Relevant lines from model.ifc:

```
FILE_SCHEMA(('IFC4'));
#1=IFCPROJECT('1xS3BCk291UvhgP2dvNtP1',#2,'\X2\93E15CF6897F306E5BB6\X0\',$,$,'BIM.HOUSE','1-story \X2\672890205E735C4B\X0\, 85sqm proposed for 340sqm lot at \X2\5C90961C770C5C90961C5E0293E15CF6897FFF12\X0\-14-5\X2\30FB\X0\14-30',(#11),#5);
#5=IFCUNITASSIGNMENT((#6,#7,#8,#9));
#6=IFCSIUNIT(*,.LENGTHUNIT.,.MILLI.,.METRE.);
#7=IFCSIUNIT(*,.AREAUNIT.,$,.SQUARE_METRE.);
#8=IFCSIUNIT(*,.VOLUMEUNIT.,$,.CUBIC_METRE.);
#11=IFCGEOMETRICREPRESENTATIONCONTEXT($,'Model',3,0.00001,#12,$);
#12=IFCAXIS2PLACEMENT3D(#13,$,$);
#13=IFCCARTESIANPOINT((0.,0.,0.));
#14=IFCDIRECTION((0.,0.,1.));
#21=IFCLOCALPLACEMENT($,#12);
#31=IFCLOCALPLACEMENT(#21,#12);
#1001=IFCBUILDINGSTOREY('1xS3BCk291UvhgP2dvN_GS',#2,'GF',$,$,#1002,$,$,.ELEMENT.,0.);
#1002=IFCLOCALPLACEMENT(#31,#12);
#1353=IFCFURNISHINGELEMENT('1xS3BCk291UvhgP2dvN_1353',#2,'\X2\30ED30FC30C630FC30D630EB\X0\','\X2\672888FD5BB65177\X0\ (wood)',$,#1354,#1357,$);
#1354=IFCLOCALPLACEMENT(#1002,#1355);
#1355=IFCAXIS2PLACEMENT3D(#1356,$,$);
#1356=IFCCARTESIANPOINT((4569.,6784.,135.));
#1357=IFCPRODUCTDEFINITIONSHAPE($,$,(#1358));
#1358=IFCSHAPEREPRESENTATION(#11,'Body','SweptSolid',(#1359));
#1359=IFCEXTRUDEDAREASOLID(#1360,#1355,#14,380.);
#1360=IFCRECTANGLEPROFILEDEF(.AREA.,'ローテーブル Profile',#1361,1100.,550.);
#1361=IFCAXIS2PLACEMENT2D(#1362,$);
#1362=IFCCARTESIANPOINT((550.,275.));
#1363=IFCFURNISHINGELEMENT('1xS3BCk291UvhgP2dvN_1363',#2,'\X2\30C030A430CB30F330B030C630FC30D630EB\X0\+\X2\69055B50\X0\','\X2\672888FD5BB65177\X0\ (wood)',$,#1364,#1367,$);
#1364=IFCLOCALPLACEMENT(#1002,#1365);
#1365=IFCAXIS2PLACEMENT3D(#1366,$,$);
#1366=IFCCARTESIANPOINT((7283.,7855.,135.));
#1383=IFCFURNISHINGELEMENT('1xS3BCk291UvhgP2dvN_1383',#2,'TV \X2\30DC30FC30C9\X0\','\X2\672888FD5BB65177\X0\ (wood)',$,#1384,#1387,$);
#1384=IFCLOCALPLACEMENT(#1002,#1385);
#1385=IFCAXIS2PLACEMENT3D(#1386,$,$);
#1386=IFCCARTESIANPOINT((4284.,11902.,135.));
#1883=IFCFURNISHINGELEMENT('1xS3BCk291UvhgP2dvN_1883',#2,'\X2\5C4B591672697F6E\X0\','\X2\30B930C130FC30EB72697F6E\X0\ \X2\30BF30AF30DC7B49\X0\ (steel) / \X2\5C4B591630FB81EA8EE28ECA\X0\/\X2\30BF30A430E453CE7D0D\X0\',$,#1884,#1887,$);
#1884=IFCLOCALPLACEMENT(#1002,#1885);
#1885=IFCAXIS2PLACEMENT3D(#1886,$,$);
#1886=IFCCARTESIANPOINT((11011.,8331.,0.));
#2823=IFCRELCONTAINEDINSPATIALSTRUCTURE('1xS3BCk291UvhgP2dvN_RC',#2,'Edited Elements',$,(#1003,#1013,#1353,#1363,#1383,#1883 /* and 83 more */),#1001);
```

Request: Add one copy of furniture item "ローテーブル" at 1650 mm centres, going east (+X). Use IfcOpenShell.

```python
import numpy as np
import ifcopenshell
import ifcopenshell.api.geometry
import ifcopenshell.api.root
import ifcopenshell.util.element
import ifcopenshell.util.placement
import ifcopenshell.util.unit

model = ifcopenshell.open("model.ifc")
unit_scale = ifcopenshell.util.unit.calculate_unit_scale(model)


def reuse_history(source, copy):
    """copy_class also copies each property set's owner history, people and application; keep the originals."""
    for rel in copy.IsDefinedBy:
        if rel.is_a("IfcRelDefinesByProperties") and (history := rel.RelatingPropertyDefinition.OwnerHistory):
            rel.RelatingPropertyDefinition.OwnerHistory = source.OwnerHistory
            ifcopenshell.util.element.remove_deep2(model, history)


source = model.by_guid("1xS3BCk291UvhgP2dvN_1353")
base = ifcopenshell.util.placement.get_local_placement(source.ObjectPlacement)
step = np.array([1.0, 0.0, 0.0]) * 1.65 / unit_scale

for i in range(1, 2):
    copy = ifcopenshell.api.root.copy_class(model, product=source)
    copy.Representation = ifcopenshell.util.element.copy_deep(
        model, source.Representation, exclude=["IfcGeometricRepresentationContext", "IfcRepresentationMap"]
    )
    reuse_history(source, copy)
    matrix = base.copy()
    matrix[:3, 3] += i * step
    print("added at", matrix[:3, 3].round(3) + 0.0)
    ifcopenshell.api.geometry.edit_object_placement(model, product=copy, matrix=matrix, is_si=False)

model.write("model_rev.ifc")
```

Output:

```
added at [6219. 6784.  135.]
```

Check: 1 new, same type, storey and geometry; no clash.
